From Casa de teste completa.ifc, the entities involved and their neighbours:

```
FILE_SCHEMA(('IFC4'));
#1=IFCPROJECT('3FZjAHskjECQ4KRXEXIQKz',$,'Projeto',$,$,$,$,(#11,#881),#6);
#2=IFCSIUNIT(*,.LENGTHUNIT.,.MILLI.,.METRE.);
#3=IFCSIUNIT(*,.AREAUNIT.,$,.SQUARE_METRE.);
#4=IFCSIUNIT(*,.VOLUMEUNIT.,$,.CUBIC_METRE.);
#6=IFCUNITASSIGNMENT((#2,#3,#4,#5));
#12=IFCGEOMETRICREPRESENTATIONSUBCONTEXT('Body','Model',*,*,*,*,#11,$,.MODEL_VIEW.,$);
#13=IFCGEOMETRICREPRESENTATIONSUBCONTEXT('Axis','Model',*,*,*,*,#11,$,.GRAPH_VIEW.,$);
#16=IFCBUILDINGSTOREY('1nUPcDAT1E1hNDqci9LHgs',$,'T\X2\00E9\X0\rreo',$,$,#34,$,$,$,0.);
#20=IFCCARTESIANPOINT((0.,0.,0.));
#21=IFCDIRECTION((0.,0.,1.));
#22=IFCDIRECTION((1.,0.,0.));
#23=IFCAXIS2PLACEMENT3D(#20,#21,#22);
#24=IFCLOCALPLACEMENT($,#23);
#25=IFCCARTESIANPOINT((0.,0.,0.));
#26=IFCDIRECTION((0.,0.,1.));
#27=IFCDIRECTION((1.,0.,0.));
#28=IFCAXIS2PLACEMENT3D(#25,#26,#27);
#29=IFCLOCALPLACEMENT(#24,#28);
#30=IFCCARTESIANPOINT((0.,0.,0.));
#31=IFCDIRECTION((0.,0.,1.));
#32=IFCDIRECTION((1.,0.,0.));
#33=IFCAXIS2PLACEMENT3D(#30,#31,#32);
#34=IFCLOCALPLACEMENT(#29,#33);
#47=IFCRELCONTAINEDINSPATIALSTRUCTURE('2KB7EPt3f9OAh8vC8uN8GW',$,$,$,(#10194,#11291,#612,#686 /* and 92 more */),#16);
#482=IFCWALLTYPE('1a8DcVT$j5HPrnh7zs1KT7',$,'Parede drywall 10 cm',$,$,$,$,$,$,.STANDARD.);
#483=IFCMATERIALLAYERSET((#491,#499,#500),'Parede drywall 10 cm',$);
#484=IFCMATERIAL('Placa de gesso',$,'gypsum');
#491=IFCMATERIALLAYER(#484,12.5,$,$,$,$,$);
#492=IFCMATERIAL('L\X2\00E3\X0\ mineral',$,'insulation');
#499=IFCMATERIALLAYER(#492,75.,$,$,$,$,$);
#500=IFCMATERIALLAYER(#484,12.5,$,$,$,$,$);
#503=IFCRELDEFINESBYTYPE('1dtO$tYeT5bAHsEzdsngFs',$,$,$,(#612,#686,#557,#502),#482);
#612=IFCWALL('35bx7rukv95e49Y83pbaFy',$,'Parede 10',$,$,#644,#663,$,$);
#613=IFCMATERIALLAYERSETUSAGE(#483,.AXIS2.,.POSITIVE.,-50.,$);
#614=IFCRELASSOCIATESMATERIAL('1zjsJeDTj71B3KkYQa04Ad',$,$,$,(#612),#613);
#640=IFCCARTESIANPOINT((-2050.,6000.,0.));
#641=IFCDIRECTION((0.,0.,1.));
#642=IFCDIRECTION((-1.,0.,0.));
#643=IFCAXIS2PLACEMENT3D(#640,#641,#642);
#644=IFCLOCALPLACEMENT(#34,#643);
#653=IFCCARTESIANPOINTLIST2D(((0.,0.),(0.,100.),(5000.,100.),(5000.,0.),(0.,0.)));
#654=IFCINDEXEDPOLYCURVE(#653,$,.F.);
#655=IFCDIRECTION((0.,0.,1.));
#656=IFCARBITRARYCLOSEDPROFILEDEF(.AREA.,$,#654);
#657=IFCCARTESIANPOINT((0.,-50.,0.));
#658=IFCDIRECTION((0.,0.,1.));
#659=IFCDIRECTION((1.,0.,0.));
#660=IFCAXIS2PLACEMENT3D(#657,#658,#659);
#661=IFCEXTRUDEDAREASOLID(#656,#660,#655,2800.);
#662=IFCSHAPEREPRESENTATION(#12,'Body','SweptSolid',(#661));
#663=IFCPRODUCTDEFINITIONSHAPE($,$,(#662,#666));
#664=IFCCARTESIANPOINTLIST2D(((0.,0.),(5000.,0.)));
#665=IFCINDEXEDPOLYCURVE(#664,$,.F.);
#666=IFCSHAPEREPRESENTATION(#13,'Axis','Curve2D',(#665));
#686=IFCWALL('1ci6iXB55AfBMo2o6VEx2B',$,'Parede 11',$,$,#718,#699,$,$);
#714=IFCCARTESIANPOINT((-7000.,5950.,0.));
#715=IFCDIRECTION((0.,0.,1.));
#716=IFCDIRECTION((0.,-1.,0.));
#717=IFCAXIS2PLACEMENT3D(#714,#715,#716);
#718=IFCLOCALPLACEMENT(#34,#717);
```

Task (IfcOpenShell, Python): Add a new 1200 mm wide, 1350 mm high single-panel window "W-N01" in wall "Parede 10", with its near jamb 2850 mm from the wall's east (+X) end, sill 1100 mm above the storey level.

```python
import numpy as np
import ifcopenshell
import ifcopenshell.api.feature
import ifcopenshell.api.geometry
import ifcopenshell.api.root
import ifcopenshell.api.spatial
import ifcopenshell.geom
import ifcopenshell.util.element
import ifcopenshell.util.placement
import ifcopenshell.util.representation
import ifcopenshell.util.shape
import ifcopenshell.util.unit

model = ifcopenshell.open("Casa de teste completa.ifc")
unit_scale = ifcopenshell.util.unit.calculate_unit_scale(model)
settings = ifcopenshell.geom.settings()


def volume(element):
    """Net volume in cubic metres, openings subtracted."""
    shape = ifcopenshell.geom.create_shape(settings, element)
    return ifcopenshell.util.shape.get_volume(shape.geometry)


wall = model.by_guid("35bx7rukv95e49Y83pbaFy")
storey = ifcopenshell.util.element.get_container(wall, ifc_class="IfcBuildingStorey")
context = ifcopenshell.util.representation.get_context(model, "Model", "Body", "MODEL_VIEW")
before = volume(wall)

width, height, from_end, sill = 1.2, 1.35, 2.85, 1.1  # metres

# The wall runs along its own X axis, and the end named is its -X end.
wall_shape = ifcopenshell.geom.create_shape(settings, wall)
x, y, z = ifcopenshell.util.shape.get_vertices(wall_shape.geometry).T
start = x.min() + from_end
face, thickness = float(y.min()), float(y.max() - y.min())
wall_matrix = ifcopenshell.util.placement.get_local_placement(wall.ObjectPlacement)
level = ifcopenshell.util.placement.get_local_placement(storey.ObjectPlacement)[2, 3]


def in_wall(x, y):
    """Placement at x, y metres in the wall's axes, at sill height."""
    matrix = wall_matrix.copy()
    matrix[:, 3] = wall_matrix @ np.array([x / unit_scale, y / unit_scale, 0.0, 1.0])
    matrix[2, 3] = level + sill / unit_scale
    return matrix


# Opening: a box that overshoots both wall faces by 50 mm.
opening = ifcopenshell.api.root.create_entity(model, ifc_class="IfcOpeningElement", predefined_type="OPENING")
box = ifcopenshell.api.geometry.add_wall_representation(
    model, context=context, length=width, height=height, thickness=thickness + 0.1
)
ifcopenshell.api.geometry.assign_representation(model, product=opening, representation=box)
ifcopenshell.api.geometry.edit_object_placement(model, product=opening, matrix=in_wall(start, face - 0.05), is_si=False)
ifcopenshell.api.feature.add_feature(model, feature=opening, element=wall)

window = ifcopenshell.api.root.create_entity(model, ifc_class="IfcWindow", name="W-N01", predefined_type="WINDOW")
window.OverallWidth, window.OverallHeight = width / unit_scale, height / unit_scale
window.PartitioningType = "SINGLE_PANEL"
body = ifcopenshell.api.geometry.add_window_representation(
    model,
    context=context,
    overall_width=window.OverallWidth,
    overall_height=window.OverallHeight,
    partition_type="SINGLE_PANEL",
)
ifcopenshell.api.geometry.assign_representation(model, product=window, representation=body)
ifcopenshell.api.spatial.assign_container(model, products=[window], relating_structure=storey)
ifcopenshell.api.feature.add_filling(model, opening=opening, element=window)

# Centre the window in the wall's thickness.
ifcopenshell.api.geometry.edit_object_placement(model, product=window, matrix=in_wall(start, face), is_si=False)
window_shape = ifcopenshell.geom.create_shape(settings, window)
depth = ifcopenshell.util.shape.get_vertices(window_shape.geometry)[:, 1]
offset = face + thickness / 2 - (depth.min() + depth.max()) / 2
ifcopenshell.api.geometry.edit_object_placement(model, product=window, matrix=in_wall(start, offset), is_si=False)

after = volume(wall)

print(f"wall volume {before:.3f} -> {after:.3f} m3")

model.write("Casa de teste completa_v2.ifc")
```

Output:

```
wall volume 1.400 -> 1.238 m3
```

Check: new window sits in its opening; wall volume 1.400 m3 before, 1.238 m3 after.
